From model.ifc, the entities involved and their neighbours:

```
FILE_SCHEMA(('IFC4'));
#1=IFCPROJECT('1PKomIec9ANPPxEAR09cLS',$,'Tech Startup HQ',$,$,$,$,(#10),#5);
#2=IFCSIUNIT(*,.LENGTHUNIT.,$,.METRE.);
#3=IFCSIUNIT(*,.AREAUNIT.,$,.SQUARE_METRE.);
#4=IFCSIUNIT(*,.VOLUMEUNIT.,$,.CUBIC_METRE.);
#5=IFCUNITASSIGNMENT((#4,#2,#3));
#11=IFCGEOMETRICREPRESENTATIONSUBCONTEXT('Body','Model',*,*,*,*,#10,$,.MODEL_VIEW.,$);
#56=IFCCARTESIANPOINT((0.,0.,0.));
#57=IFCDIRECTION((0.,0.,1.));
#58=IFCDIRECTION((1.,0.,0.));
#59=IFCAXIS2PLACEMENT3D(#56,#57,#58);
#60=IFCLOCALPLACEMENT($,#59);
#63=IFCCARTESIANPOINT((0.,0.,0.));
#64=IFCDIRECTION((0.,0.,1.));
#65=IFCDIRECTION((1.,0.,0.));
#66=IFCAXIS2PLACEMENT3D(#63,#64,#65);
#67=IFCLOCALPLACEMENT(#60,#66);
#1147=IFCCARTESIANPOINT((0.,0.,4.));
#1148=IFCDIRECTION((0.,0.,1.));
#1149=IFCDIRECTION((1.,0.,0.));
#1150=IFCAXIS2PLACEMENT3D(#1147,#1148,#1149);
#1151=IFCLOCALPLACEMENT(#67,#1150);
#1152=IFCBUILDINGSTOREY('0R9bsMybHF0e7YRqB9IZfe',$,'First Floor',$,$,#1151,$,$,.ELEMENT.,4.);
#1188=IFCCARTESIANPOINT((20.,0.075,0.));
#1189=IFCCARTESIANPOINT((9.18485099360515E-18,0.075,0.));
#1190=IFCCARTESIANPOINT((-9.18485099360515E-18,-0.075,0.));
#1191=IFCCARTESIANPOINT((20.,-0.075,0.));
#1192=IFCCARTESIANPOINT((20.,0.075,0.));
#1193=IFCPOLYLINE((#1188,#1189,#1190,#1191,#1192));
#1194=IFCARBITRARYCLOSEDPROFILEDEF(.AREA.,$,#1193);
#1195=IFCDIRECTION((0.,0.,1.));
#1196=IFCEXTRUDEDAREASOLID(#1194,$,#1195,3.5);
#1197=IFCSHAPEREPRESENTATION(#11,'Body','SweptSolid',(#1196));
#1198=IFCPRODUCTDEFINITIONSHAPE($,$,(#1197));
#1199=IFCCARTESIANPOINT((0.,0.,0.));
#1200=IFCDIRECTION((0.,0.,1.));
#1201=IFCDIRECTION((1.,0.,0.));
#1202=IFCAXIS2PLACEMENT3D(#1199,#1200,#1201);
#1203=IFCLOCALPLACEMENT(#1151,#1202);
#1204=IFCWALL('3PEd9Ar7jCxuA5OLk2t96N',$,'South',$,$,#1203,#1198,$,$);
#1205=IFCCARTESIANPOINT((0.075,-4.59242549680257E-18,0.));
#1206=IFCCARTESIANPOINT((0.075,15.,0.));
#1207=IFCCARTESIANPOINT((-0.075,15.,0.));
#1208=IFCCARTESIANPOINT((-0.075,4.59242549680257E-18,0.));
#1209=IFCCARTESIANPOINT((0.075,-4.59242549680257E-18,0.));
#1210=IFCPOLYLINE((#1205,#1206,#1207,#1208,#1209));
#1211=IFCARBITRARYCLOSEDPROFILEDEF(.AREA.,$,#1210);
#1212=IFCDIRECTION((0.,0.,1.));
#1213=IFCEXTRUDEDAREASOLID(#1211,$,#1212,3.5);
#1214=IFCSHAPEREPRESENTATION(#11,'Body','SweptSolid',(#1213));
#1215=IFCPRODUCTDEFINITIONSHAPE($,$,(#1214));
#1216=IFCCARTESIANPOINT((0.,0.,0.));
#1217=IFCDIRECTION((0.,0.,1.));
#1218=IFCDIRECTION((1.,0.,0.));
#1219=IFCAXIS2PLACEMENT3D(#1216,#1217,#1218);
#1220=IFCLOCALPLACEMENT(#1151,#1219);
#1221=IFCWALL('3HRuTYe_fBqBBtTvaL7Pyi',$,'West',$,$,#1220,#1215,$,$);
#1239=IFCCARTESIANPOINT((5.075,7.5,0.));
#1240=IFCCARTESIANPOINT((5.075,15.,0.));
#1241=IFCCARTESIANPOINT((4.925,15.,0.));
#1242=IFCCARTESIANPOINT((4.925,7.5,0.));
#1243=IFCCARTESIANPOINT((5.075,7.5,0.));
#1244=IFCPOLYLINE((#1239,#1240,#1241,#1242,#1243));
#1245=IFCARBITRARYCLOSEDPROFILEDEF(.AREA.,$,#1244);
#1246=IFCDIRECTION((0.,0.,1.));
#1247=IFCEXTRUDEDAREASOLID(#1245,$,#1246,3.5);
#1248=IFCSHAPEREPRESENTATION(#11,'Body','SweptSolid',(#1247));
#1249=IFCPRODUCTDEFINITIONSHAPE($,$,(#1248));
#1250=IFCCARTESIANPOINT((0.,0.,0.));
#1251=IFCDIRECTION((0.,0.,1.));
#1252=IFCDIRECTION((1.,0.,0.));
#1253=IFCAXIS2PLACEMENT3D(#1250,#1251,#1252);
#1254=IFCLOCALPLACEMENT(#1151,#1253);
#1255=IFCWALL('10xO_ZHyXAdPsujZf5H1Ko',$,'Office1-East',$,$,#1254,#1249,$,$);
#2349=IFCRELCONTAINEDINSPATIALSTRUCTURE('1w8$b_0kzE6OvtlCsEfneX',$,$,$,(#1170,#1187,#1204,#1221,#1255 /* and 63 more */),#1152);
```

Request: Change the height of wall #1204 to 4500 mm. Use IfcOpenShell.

```python
import ifcopenshell
import ifcopenshell.geom
import ifcopenshell.util.representation
import ifcopenshell.util.shape
import ifcopenshell.util.unit

model = ifcopenshell.open("model.ifc")
unit_scale = ifcopenshell.util.unit.calculate_unit_scale(model)
settings = ifcopenshell.geom.settings()


def volume(element):
    """Net volume in cubic metres, openings subtracted."""
    shape = ifcopenshell.geom.create_shape(settings, element)
    return ifcopenshell.util.shape.get_volume(shape.geometry)


wall = model.by_guid("3PEd9Ar7jCxuA5OLk2t96N")
before = volume(wall)

body = ifcopenshell.util.representation.get_representation(wall, "Model", "Body")
solid = body.Items[0]
old_height = solid.Depth
solid.Depth = 4.5 / unit_scale
after = volume(wall)

print(f"height {old_height:g} -> {solid.Depth:g}, volume {before:.3f} -> {after:.3f} m3")

model.write("model_updated.ifc")
```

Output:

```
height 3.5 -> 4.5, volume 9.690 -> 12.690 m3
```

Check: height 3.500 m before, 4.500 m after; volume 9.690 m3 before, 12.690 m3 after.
